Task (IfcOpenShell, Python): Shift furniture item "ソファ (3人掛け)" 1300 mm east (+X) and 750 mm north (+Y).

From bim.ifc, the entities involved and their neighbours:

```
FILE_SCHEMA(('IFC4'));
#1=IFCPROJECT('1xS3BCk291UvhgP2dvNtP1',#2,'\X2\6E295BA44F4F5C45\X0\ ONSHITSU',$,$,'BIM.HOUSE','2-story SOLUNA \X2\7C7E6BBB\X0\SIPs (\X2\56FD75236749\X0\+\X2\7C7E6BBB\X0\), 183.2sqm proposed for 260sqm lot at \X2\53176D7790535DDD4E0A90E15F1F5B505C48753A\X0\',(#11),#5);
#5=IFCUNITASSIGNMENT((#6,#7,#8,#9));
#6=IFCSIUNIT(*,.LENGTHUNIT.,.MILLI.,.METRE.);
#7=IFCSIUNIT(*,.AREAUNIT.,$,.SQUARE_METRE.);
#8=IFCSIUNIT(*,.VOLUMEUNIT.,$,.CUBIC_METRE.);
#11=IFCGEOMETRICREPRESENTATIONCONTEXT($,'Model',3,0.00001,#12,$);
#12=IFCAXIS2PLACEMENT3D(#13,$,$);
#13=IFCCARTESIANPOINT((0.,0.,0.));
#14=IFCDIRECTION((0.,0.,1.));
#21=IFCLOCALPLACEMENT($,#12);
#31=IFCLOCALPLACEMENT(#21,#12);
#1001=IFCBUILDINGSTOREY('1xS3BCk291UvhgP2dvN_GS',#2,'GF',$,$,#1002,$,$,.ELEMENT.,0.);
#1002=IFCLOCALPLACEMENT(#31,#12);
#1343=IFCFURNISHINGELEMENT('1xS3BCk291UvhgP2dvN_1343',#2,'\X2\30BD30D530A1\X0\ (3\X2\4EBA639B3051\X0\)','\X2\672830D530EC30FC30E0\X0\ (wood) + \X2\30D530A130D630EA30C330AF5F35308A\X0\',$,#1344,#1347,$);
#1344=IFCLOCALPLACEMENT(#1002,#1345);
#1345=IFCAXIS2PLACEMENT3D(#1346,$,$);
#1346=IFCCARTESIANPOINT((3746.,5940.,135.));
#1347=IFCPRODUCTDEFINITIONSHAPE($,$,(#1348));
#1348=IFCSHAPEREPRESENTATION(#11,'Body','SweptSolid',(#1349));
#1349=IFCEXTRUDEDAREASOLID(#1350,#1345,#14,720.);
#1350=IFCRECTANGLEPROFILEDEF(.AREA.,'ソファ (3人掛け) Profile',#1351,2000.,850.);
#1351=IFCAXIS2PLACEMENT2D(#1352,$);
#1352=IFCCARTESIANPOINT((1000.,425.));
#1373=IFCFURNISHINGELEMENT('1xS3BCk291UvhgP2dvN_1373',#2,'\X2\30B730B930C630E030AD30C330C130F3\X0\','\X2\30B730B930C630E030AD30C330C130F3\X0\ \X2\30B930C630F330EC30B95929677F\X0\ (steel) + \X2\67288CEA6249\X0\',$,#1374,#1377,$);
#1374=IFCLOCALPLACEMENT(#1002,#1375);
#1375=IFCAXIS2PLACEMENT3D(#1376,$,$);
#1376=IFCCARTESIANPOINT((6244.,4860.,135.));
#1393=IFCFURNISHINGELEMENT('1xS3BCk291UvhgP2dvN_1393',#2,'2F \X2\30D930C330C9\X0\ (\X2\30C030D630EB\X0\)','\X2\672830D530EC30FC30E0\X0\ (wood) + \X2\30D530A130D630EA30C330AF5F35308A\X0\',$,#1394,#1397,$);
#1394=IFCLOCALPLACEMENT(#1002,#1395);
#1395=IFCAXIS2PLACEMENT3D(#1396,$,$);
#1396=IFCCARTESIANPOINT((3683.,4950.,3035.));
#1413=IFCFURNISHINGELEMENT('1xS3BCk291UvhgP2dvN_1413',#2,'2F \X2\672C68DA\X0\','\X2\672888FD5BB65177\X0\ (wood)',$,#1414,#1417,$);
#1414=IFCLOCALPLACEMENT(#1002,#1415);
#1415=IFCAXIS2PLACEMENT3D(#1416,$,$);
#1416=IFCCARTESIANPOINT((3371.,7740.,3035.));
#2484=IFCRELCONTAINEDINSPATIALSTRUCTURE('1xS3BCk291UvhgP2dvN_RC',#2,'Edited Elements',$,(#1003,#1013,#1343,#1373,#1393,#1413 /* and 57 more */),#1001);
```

```python
import ifcopenshell
import ifcopenshell.api.geometry
import ifcopenshell.util.placement
import ifcopenshell.util.unit

model = ifcopenshell.open("bim.ifc")
unit_scale = ifcopenshell.util.unit.calculate_unit_scale(model)

item = model.by_guid("1xS3BCk291UvhgP2dvN_1343")
matrix = ifcopenshell.util.placement.get_local_placement(item.ObjectPlacement)
matrix[0, 3] += 1.3 / unit_scale
matrix[1, 3] += 0.75 / unit_scale
ifcopenshell.api.geometry.edit_object_placement(model, product=item, matrix=matrix, is_si=False)

print(ifcopenshell.util.placement.get_local_placement(item.ObjectPlacement).round(3) + 0.0)

model.write("bim_v2.ifc")
```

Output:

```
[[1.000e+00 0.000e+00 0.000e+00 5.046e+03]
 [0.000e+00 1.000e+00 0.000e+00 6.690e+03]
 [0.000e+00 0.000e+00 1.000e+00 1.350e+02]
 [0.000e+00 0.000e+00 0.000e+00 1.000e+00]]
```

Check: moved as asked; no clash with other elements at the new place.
